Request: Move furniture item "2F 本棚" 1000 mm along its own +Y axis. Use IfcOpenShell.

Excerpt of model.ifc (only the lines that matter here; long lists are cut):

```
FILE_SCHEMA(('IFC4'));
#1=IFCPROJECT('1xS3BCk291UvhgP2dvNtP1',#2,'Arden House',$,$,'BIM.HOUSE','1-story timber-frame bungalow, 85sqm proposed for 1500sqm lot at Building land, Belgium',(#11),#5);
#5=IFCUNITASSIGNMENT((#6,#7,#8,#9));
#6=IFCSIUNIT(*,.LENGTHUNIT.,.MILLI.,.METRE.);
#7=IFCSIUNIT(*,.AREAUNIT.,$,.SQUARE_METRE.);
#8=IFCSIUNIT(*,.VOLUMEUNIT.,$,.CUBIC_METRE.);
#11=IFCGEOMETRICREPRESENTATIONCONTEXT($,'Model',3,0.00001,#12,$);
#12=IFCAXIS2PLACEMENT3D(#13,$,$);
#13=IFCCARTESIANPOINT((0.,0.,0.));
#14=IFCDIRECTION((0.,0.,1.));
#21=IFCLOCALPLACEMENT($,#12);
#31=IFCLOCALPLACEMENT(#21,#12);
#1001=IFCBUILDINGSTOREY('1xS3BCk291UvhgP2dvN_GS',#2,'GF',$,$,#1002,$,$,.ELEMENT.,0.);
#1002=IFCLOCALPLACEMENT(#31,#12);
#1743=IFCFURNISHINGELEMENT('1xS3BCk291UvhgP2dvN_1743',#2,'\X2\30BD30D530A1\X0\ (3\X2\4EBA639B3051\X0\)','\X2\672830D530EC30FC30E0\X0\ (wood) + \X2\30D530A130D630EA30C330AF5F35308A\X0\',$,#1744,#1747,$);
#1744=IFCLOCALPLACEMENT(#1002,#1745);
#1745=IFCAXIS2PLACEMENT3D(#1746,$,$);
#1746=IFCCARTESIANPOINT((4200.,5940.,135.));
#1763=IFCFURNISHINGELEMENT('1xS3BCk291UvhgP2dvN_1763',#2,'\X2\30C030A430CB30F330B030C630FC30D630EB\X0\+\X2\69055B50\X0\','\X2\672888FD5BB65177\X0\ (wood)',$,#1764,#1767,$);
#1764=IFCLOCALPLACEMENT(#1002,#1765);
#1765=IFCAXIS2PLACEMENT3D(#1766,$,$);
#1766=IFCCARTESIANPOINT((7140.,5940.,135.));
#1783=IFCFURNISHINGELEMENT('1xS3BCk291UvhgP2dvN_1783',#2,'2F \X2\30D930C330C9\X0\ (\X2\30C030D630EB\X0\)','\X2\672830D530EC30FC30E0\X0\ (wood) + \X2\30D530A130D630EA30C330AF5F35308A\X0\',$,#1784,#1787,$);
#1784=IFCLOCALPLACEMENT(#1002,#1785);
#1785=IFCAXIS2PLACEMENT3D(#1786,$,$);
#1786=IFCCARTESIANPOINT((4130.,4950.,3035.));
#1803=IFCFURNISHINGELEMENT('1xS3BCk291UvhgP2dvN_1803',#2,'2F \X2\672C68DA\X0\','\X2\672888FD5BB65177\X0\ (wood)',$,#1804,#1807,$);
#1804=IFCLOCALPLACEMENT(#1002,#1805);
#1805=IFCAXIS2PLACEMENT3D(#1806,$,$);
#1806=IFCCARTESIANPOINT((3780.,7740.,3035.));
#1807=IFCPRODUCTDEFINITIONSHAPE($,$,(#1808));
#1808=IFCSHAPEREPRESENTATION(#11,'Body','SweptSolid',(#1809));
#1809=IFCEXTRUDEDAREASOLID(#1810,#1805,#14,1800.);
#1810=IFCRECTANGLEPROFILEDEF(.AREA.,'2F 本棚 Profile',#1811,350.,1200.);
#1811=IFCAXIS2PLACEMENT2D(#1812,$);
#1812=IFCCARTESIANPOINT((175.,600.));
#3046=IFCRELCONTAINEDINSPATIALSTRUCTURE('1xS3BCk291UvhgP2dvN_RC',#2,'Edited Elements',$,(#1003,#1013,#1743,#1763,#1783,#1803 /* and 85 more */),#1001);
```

```python
import ifcopenshell
import ifcopenshell.api.geometry
import ifcopenshell.util.placement

model = ifcopenshell.open("model.ifc")

item = model.by_guid("1xS3BCk291UvhgP2dvN_1803")
matrix = ifcopenshell.util.placement.get_local_placement(item.ObjectPlacement)
matrix[:3, 3] += matrix[:3, 1] * 1000.0
ifcopenshell.api.geometry.edit_object_placement(model, product=item, matrix=matrix, is_si=False)

print(ifcopenshell.util.placement.get_local_placement(item.ObjectPlacement).round(3) + 0.0)

model.write("model_edited.ifc")
```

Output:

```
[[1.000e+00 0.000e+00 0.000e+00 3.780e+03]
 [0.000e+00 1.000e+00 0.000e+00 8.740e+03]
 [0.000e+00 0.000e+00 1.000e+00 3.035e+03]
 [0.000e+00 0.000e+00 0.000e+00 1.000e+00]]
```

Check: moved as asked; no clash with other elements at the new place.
